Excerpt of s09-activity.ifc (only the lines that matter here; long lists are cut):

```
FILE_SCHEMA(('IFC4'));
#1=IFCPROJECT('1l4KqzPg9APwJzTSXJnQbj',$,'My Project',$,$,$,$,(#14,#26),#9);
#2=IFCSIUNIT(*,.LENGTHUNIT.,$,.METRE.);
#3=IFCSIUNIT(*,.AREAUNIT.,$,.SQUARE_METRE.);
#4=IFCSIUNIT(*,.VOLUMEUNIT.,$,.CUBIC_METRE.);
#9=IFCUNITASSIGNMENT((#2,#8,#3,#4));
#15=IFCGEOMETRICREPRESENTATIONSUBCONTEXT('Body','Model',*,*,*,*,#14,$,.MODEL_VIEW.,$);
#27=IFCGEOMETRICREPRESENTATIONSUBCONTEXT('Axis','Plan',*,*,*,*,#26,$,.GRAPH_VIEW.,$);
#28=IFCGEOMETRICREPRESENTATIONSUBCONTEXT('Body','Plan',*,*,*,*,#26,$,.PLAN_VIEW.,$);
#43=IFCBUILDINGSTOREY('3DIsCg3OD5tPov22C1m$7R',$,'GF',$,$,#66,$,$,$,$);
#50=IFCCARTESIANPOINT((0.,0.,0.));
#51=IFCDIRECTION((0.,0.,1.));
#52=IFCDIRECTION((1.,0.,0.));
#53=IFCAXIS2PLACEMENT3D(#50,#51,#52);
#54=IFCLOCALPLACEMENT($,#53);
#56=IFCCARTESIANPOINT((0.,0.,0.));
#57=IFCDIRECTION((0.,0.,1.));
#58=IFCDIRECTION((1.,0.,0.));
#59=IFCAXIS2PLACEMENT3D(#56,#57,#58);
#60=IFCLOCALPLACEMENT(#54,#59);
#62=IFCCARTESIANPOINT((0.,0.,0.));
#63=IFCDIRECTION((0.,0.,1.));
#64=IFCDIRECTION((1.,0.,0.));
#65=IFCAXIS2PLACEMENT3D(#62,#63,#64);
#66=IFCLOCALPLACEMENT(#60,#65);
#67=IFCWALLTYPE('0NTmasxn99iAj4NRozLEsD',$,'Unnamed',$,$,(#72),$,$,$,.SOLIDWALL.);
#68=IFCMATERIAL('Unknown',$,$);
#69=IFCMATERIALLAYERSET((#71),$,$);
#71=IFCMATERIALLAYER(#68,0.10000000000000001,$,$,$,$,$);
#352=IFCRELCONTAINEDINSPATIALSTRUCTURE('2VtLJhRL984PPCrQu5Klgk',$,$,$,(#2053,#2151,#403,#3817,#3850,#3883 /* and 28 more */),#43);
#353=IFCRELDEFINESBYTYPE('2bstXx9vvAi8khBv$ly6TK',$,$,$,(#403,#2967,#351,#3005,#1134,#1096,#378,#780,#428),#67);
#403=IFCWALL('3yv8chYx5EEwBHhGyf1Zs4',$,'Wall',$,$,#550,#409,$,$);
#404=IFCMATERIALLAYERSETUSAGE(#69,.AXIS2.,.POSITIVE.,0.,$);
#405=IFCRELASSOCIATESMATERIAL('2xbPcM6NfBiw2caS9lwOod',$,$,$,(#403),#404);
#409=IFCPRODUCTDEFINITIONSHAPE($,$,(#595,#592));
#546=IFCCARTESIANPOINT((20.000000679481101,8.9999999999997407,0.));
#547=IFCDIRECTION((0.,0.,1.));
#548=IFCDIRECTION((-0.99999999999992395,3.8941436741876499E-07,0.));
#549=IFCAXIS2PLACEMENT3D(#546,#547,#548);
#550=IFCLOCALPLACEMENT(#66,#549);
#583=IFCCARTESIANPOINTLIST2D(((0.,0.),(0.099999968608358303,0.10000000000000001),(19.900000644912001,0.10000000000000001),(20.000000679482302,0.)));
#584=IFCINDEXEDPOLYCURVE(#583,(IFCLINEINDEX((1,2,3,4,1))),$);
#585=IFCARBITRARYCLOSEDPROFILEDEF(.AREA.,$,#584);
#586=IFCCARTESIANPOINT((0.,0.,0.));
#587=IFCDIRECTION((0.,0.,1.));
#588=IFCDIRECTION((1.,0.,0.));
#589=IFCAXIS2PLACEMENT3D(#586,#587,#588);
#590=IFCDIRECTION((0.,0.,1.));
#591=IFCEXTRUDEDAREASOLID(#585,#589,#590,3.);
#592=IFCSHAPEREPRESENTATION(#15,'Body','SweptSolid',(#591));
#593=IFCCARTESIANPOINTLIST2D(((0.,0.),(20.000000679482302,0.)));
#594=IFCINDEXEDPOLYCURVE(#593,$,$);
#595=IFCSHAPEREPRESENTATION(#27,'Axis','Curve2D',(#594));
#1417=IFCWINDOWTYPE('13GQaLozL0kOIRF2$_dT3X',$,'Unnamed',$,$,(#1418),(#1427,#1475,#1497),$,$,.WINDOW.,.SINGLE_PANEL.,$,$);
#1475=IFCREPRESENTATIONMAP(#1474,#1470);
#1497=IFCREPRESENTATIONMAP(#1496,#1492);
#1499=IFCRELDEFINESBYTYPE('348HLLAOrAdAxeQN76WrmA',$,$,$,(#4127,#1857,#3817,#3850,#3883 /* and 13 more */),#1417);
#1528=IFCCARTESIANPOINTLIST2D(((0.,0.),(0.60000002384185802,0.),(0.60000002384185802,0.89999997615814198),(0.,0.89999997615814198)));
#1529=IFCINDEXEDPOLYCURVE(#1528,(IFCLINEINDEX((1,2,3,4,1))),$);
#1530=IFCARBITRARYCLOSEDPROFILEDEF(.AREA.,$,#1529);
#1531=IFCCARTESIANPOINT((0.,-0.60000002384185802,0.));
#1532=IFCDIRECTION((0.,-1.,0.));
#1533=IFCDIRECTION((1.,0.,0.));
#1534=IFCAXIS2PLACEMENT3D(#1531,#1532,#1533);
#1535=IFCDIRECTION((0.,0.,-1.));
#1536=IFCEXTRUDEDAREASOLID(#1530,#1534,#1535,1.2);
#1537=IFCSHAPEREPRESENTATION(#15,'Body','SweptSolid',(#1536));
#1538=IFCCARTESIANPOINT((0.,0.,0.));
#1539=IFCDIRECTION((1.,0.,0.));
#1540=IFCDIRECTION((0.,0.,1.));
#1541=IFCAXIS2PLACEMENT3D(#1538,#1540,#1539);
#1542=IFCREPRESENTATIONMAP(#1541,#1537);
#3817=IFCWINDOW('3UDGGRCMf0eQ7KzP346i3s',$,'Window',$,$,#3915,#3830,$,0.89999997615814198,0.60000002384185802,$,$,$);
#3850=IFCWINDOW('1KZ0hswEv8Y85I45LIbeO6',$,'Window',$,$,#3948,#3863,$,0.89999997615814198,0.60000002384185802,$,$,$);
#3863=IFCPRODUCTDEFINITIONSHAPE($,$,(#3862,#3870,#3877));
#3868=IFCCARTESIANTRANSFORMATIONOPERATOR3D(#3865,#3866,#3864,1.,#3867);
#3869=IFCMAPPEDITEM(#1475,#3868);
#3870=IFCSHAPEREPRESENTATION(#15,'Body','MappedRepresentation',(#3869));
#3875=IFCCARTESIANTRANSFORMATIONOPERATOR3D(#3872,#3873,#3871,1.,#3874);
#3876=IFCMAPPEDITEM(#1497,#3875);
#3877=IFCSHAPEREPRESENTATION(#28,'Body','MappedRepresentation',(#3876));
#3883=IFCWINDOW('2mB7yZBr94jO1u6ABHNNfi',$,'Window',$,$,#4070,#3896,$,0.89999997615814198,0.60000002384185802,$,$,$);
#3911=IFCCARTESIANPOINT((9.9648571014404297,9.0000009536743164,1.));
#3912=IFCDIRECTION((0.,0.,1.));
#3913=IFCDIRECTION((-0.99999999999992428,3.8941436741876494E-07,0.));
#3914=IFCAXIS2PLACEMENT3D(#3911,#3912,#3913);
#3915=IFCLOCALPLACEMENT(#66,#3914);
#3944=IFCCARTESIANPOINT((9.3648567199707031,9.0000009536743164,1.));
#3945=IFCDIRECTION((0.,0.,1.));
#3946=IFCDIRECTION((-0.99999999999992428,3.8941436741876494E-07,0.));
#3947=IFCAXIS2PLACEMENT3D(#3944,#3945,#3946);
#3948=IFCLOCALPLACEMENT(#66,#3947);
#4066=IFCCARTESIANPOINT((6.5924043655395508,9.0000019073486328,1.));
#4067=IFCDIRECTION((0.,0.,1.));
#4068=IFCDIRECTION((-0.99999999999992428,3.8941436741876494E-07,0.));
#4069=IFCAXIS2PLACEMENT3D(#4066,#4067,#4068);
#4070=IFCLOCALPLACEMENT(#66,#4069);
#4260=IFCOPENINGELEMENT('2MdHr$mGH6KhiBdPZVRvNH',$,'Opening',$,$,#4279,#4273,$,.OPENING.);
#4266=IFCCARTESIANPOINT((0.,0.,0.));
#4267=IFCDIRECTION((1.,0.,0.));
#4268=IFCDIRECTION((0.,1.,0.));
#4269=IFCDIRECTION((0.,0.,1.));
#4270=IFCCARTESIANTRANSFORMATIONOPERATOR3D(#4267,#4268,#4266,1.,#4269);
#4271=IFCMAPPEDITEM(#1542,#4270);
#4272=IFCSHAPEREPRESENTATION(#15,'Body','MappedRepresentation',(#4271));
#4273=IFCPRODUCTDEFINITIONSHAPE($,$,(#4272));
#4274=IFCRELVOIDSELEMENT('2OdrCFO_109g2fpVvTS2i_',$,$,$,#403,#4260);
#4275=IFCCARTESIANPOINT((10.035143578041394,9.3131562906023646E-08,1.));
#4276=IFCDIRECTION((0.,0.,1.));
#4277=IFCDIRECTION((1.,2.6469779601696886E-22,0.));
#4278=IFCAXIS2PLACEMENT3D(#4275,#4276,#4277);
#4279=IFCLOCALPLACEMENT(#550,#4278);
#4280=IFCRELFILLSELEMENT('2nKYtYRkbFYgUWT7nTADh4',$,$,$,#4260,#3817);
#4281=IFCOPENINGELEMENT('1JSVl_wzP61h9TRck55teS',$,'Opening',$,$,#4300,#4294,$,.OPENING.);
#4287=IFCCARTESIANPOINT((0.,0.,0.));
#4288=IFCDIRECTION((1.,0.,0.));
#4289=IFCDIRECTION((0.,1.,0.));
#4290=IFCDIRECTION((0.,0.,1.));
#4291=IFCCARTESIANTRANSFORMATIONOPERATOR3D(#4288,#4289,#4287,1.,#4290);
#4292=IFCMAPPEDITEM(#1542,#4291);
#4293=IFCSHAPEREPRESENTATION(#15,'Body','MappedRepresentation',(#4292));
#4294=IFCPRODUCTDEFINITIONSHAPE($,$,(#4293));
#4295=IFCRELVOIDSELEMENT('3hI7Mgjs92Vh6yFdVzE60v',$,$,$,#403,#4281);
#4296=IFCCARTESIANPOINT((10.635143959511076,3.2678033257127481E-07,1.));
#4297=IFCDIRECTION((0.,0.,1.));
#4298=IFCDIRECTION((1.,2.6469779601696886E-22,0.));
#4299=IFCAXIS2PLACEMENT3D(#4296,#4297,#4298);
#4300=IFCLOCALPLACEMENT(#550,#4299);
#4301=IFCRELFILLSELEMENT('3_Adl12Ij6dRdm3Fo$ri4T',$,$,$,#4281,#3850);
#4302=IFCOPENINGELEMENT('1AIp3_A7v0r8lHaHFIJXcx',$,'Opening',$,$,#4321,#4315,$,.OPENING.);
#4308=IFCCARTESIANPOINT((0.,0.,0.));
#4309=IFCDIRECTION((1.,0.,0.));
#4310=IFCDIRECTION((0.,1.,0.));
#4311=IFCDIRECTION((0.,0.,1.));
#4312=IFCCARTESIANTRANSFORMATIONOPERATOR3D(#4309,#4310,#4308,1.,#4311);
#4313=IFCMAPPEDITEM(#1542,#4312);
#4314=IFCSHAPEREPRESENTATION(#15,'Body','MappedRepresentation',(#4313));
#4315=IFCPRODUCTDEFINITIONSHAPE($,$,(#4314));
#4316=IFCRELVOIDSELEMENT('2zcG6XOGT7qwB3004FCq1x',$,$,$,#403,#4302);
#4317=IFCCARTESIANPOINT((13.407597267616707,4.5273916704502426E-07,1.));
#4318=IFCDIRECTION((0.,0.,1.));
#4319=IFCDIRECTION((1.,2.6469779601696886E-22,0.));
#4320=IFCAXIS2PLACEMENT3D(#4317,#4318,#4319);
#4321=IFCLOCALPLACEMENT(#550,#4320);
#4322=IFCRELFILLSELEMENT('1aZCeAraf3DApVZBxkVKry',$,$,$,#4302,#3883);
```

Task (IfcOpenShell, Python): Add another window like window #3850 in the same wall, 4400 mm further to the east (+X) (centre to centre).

```python
import ifcopenshell
import ifcopenshell.api.feature
import ifcopenshell.api.geometry
import ifcopenshell.api.root
import ifcopenshell.geom
import ifcopenshell.util.element
import ifcopenshell.util.placement
import ifcopenshell.util.shape
import ifcopenshell.util.unit

model = ifcopenshell.open("s09-activity.ifc")
unit_scale = ifcopenshell.util.unit.calculate_unit_scale(model)
settings = ifcopenshell.geom.settings()


def volume(element):
    """Net volume in cubic metres, openings subtracted."""
    shape = ifcopenshell.geom.create_shape(settings, element)
    return ifcopenshell.util.shape.get_volume(shape.geometry)


window = model.by_guid("1KZ0hswEv8Y85I45LIbeO6")
opening = window.FillsVoids[0].RelatingOpeningElement
wall = opening.VoidsElements[0].RelatingBuildingElement
before = volume(wall)
shift = ifcopenshell.util.placement.get_local_placement(wall.ObjectPlacement)[:3, 0] * -4.4 / unit_scale

# copy_class copies the void relationship, type, container and properties, but no geometry.
new_opening = ifcopenshell.api.root.copy_class(model, product=opening)
new_opening.Representation = ifcopenshell.util.element.copy_deep(
    model, opening.Representation, exclude=["IfcGeometricRepresentationContext", "IfcRepresentationMap"]
)
new_window = ifcopenshell.api.root.copy_class(model, product=window)
new_window.Representation = ifcopenshell.util.element.copy_deep(
    model, window.Representation, exclude=["IfcGeometricRepresentationContext", "IfcRepresentationMap"]
)
ifcopenshell.api.feature.add_filling(model, opening=new_opening, element=new_window)

for old, new in ((opening, new_opening), (window, new_window)):
    matrix = ifcopenshell.util.placement.get_local_placement(old.ObjectPlacement)
    matrix[:3, 3] += shift
    ifcopenshell.api.geometry.edit_object_placement(model, product=new, matrix=matrix, is_si=False)

after = volume(wall)

print(f"wall volume {before:.3f} -> {after:.3f} m3")

model.write("s09-activity_edited.ifc")
```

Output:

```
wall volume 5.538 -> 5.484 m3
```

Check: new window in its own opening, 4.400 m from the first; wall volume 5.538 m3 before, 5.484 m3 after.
